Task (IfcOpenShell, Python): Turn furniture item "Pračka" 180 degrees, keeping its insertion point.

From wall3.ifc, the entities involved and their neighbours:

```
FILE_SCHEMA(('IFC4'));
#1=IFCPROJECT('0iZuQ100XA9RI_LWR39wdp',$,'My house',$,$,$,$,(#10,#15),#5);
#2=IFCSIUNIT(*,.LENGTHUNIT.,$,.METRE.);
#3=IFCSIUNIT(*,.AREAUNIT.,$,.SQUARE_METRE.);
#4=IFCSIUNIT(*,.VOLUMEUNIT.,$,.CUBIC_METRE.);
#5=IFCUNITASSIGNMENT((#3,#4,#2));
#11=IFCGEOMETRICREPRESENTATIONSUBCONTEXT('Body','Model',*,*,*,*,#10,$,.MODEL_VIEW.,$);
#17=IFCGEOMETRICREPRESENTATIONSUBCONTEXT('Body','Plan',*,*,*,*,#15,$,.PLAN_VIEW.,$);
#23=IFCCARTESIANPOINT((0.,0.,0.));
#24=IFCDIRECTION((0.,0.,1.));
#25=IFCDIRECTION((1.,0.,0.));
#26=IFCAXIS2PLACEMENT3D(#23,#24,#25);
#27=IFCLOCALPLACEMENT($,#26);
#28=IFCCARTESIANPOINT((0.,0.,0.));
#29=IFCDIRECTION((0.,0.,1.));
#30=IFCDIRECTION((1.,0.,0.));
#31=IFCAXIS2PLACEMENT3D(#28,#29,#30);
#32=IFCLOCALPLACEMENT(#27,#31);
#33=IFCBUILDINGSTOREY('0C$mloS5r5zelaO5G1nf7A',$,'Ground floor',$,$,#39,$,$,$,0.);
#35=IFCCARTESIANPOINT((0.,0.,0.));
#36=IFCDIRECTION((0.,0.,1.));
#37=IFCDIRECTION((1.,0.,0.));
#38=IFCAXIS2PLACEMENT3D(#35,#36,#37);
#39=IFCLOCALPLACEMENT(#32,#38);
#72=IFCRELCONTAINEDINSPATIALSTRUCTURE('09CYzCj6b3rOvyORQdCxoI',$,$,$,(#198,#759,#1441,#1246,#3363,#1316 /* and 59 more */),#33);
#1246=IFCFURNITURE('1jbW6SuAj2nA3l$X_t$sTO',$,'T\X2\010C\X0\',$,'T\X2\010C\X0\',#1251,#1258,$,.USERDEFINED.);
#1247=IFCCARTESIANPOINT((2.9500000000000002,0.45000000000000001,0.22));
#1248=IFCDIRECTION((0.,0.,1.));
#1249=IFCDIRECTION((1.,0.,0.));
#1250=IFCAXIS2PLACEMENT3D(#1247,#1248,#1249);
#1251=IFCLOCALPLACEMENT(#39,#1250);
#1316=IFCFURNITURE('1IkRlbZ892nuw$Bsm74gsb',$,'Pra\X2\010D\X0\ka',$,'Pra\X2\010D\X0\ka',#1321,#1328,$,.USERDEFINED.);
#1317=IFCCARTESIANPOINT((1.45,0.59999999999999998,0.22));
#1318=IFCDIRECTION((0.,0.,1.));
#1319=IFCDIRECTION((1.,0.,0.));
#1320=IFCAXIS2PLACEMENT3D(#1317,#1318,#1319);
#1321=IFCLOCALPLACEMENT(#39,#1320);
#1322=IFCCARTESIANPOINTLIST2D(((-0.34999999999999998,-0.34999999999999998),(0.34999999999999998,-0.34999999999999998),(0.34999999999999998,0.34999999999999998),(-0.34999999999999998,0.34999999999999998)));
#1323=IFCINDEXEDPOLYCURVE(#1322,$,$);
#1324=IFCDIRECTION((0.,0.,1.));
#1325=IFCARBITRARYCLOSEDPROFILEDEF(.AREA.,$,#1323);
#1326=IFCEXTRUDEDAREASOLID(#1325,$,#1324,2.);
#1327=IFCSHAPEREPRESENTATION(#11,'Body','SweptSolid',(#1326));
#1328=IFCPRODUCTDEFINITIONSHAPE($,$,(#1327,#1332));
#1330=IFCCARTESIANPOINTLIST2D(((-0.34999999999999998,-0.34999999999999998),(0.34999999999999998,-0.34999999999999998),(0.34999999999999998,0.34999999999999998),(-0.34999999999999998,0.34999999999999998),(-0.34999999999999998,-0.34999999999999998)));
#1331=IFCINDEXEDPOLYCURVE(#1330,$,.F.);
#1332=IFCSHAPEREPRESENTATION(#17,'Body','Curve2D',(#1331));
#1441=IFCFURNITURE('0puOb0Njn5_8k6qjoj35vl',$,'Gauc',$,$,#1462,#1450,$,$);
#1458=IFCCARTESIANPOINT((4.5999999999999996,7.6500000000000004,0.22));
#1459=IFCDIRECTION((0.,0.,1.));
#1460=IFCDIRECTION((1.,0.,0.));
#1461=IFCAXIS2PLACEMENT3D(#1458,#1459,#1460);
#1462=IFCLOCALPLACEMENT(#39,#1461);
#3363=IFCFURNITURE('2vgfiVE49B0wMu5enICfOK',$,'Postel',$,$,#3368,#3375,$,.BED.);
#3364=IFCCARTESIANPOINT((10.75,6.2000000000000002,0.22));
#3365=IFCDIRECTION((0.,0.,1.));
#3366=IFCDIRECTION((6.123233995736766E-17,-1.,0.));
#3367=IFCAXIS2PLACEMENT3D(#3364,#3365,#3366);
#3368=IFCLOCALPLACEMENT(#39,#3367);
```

```python
import ifcopenshell
import ifcopenshell.api.geometry
import ifcopenshell.util.placement

model = ifcopenshell.open("wall3.ifc")

item = model.by_id(1316)
matrix = ifcopenshell.util.placement.get_local_placement(item.ObjectPlacement)
matrix = matrix @ ifcopenshell.util.placement.rotation(180, "Z")
ifcopenshell.api.geometry.edit_object_placement(model, product=item, matrix=matrix, is_si=False)

print(ifcopenshell.util.placement.get_local_placement(item.ObjectPlacement).round(3) + 0.0)

model.write("wall3-out.ifc")
```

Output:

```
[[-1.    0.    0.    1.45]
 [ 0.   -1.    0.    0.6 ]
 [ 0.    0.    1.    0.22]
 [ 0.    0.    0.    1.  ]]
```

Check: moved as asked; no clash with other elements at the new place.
